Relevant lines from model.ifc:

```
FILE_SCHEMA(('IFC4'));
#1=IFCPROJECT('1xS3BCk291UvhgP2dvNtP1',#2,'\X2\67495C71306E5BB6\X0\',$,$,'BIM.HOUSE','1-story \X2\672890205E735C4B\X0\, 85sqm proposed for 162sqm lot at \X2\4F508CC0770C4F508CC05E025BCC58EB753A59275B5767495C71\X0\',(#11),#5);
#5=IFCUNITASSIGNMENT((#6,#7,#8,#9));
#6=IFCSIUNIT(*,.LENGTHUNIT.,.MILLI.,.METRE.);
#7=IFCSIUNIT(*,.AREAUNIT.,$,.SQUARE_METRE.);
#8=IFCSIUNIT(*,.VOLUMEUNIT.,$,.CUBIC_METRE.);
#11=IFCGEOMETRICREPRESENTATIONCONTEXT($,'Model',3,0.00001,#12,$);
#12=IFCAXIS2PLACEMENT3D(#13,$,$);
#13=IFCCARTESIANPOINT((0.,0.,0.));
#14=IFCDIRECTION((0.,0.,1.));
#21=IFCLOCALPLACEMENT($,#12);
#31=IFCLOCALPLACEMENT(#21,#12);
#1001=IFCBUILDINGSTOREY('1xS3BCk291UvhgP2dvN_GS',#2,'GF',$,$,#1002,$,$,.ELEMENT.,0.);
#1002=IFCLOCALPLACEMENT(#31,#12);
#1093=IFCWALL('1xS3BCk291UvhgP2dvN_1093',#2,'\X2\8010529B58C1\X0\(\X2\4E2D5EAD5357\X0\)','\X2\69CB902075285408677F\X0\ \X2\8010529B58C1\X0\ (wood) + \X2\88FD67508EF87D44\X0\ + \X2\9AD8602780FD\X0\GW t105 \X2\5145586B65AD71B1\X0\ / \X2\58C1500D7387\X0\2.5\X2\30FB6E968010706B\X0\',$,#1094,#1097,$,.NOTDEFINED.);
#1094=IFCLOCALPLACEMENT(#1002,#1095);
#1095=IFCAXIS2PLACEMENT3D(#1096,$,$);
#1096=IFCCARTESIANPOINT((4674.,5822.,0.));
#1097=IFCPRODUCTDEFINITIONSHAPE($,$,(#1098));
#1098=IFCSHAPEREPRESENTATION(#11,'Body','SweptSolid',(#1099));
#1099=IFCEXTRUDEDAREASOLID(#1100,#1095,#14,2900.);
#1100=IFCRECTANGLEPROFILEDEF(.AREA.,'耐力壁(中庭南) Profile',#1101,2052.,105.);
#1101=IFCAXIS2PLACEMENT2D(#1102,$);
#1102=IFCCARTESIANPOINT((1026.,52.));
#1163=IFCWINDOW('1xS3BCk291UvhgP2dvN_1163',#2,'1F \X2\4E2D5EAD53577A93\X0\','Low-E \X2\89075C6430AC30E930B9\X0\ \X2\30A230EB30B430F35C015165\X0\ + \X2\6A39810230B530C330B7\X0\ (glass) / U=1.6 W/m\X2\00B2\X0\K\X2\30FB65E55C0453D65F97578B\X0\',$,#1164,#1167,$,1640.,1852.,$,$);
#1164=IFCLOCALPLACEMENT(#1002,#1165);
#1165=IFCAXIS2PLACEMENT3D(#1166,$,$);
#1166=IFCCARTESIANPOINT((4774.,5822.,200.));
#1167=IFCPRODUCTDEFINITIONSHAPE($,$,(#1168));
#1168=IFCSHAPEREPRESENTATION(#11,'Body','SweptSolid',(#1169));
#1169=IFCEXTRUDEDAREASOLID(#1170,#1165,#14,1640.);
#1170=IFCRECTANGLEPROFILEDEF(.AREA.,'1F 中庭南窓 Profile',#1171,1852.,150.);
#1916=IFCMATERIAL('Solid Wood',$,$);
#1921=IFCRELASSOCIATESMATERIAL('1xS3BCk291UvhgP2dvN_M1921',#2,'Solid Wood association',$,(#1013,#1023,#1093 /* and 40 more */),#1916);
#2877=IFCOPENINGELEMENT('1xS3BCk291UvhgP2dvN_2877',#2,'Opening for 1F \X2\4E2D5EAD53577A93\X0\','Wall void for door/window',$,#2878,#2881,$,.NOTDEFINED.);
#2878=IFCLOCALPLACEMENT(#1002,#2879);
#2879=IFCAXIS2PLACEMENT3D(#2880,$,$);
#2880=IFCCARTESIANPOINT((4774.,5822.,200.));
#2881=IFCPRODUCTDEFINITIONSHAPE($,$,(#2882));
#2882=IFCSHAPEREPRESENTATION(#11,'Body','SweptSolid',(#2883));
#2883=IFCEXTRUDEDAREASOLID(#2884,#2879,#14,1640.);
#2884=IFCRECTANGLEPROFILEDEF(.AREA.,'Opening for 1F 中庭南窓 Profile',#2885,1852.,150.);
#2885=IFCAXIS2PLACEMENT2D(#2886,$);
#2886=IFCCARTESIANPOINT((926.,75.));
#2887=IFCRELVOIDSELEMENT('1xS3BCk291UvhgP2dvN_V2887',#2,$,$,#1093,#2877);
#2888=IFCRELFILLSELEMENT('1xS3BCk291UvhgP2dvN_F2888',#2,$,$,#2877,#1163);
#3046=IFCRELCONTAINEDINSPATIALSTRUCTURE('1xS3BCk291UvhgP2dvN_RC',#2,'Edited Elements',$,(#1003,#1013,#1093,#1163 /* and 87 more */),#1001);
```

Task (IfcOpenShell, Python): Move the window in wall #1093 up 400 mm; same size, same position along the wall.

```python
import numpy as np
import ifcopenshell
import ifcopenshell.api.geometry
import ifcopenshell.util.placement
import ifcopenshell.util.unit

model = ifcopenshell.open("model.ifc")
unit_scale = ifcopenshell.util.unit.calculate_unit_scale(model)

window = model.by_guid("1xS3BCk291UvhgP2dvN_1163")
opening = window.FillsVoids[0].RelatingOpeningElement
dz = 400.0

shift = np.array([0.0, 0.0, dz])
# The window is not placed relative to its opening, so move both.
for product in (opening, window):
    matrix = ifcopenshell.util.placement.get_local_placement(product.ObjectPlacement)
    matrix[:3, 3] += shift
    ifcopenshell.api.geometry.edit_object_placement(model, product=product, matrix=matrix, is_si=False)

print(f"moved by {dz * unit_scale:+.3f} m")

model.write("model_rev.ifc")
```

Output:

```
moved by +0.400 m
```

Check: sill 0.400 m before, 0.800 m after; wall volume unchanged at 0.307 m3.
